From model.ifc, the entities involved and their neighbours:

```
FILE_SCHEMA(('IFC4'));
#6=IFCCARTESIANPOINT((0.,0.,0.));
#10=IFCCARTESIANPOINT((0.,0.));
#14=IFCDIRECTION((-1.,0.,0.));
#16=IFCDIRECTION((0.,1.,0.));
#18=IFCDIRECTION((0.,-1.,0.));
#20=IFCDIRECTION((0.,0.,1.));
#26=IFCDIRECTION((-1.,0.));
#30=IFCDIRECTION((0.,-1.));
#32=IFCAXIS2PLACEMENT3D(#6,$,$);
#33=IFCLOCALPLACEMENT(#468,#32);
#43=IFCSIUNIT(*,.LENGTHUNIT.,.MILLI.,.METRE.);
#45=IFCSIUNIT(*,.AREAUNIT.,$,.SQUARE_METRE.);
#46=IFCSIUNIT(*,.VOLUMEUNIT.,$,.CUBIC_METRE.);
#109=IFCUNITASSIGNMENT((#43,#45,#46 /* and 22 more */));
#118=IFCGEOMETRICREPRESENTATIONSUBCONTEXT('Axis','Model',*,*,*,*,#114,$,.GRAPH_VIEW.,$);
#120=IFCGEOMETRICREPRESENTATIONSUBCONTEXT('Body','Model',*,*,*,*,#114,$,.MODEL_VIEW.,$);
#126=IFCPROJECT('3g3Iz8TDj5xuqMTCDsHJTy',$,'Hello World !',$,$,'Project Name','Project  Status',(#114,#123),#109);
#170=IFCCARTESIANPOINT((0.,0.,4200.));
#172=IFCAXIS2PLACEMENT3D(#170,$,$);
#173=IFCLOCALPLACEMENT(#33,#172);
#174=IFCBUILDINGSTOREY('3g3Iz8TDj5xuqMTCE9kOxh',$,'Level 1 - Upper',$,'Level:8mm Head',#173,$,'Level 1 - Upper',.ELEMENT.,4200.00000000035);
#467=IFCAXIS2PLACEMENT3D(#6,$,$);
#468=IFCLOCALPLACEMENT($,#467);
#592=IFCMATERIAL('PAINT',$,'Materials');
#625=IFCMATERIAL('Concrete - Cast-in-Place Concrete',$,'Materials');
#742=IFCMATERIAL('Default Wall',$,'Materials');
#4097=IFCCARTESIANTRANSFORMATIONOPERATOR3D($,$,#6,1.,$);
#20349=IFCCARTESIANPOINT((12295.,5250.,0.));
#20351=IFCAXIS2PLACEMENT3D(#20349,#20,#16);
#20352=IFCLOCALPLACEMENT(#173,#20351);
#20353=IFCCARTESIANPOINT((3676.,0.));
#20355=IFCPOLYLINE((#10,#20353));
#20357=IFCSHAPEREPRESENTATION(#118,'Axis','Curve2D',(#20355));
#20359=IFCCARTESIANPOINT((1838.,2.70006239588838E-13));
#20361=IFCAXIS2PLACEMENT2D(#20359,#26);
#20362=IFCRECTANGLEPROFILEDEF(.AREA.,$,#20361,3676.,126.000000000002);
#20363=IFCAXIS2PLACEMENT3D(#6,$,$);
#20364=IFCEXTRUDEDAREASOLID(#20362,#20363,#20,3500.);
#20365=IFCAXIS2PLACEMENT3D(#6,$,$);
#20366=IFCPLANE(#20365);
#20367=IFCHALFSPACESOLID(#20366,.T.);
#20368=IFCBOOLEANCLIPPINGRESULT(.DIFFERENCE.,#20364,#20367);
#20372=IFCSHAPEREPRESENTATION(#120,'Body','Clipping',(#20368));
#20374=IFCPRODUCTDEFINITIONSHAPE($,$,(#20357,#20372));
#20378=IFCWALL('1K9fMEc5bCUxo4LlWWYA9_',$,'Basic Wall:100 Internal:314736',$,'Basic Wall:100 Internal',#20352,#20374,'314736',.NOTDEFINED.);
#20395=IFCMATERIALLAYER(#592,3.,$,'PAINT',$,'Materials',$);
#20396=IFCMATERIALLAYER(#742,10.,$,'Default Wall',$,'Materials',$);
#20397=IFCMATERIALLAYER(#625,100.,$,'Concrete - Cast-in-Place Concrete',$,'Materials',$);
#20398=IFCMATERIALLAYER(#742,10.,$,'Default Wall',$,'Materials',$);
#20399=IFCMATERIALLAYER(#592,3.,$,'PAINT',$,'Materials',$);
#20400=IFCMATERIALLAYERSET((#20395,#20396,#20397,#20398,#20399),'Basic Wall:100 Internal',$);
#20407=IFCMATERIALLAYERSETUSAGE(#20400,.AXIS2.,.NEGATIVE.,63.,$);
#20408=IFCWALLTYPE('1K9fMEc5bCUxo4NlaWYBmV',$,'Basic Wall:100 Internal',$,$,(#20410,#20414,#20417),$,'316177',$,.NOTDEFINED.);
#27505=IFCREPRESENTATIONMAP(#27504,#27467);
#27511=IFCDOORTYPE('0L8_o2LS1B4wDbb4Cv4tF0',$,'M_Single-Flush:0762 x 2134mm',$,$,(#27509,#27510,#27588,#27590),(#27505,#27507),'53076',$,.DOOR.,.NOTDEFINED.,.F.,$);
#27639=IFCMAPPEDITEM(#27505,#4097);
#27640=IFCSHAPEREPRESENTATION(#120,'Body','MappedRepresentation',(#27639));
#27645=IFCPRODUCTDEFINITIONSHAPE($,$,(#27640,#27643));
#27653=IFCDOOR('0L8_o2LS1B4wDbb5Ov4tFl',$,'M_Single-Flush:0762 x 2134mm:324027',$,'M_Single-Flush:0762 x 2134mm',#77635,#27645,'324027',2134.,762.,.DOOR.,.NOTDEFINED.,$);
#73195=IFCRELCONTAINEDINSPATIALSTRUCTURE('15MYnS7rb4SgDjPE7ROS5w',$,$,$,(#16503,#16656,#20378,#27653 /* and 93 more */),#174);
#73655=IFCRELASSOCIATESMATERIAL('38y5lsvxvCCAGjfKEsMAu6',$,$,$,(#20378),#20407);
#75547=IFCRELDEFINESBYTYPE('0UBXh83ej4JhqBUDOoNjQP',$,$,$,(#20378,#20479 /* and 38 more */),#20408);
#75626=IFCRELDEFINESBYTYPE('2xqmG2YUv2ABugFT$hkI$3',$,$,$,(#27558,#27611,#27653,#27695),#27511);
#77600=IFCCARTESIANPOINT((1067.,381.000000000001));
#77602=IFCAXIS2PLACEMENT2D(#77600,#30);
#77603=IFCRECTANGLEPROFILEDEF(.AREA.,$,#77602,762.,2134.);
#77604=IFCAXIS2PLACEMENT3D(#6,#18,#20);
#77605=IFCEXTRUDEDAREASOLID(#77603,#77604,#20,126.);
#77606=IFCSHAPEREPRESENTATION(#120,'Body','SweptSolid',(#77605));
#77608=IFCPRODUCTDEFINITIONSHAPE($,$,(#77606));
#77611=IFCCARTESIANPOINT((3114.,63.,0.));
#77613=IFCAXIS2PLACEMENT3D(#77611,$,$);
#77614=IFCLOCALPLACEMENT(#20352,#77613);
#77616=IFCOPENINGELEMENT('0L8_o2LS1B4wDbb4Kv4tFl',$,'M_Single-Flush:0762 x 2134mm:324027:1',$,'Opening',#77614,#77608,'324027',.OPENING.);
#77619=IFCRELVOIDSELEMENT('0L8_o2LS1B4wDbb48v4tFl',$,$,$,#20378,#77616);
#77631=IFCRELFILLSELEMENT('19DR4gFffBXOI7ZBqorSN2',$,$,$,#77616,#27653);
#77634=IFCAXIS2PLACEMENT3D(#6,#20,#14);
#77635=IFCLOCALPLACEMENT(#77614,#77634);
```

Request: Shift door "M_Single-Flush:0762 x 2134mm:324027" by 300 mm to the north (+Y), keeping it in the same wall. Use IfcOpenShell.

```python
import ifcopenshell
import ifcopenshell.api.geometry
import ifcopenshell.util.placement

model = ifcopenshell.open("model.ifc")

door = model.by_id(27653)
opening = door.FillsVoids[0].RelatingOpeningElement
wall = opening.VoidsElements[0].RelatingBuildingElement

wall_matrix = ifcopenshell.util.placement.get_local_placement(wall.ObjectPlacement)
shift = wall_matrix[:3, 0] * 300.0
before = ifcopenshell.util.placement.get_local_placement(door.ObjectPlacement)[:3, 3].copy()

# The door is placed relative to its opening, so it follows when the opening moves.
matrix = ifcopenshell.util.placement.get_local_placement(opening.ObjectPlacement)
matrix[:3, 3] += shift
ifcopenshell.api.geometry.edit_object_placement(
    model, product=opening, matrix=matrix, is_si=False, should_transform_children=True
)

after = ifcopenshell.util.placement.get_local_placement(door.ObjectPlacement)[:3, 3]
print("door moved by", (after - before).round(3) + 0.0)

model.write("model_v2.ifc")
```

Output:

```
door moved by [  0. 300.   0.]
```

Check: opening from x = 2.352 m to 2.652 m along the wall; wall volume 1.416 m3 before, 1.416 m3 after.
